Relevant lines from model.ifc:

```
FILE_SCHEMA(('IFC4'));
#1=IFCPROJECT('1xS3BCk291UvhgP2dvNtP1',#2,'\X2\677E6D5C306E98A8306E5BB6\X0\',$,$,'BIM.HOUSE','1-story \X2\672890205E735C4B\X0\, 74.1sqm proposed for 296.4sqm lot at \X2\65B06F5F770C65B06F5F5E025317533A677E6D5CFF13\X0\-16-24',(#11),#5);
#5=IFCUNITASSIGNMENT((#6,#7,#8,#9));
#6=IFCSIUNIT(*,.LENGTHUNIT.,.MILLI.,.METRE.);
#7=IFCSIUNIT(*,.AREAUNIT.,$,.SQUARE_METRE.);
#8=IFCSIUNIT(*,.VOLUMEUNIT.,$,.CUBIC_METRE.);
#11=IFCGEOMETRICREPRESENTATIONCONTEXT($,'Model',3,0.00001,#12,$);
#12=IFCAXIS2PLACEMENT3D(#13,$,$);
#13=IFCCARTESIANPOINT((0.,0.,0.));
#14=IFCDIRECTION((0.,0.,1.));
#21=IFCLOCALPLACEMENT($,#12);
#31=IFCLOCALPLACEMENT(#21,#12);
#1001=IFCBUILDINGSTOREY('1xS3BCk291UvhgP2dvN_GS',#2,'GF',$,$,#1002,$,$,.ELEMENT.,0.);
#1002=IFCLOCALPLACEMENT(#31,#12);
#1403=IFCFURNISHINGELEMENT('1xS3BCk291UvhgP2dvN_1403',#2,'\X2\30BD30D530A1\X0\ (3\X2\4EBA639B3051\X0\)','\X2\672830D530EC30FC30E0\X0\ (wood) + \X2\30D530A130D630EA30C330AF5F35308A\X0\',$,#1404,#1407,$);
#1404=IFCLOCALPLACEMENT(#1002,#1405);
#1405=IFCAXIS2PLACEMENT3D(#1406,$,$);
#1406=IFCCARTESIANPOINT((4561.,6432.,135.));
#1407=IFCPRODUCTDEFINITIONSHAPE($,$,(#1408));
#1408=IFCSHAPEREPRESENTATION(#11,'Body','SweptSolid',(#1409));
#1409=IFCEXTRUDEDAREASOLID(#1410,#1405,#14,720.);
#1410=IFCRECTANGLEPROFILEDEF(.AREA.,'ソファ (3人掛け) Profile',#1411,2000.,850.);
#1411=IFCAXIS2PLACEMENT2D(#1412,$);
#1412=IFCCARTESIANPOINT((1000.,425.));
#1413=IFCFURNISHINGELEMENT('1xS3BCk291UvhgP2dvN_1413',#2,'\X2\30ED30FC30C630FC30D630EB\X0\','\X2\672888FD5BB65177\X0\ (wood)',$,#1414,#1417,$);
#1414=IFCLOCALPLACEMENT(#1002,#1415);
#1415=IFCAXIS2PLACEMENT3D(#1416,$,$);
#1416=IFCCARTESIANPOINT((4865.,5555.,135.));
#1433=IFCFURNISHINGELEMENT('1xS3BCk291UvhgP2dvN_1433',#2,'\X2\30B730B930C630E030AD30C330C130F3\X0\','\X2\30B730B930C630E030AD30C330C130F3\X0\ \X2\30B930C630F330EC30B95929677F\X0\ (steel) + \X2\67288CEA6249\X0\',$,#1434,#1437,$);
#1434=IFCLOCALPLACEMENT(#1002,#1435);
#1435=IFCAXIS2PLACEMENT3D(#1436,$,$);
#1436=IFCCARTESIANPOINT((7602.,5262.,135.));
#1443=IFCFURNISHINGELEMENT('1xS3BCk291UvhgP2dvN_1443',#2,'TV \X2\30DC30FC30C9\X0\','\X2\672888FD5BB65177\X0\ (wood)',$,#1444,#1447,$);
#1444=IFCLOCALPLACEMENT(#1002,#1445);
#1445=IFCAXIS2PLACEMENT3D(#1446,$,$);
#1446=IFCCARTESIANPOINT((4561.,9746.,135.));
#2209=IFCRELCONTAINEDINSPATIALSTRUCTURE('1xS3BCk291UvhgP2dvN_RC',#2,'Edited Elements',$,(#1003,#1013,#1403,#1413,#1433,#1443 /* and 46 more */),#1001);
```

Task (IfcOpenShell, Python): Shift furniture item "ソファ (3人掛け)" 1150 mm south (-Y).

```python
import ifcopenshell
import ifcopenshell.api.geometry
import ifcopenshell.util.placement

model = ifcopenshell.open("model.ifc")

item = model.by_id(1403)
matrix = ifcopenshell.util.placement.get_local_placement(item.ObjectPlacement)
matrix[1, 3] -= 1150.0
ifcopenshell.api.geometry.edit_object_placement(model, product=item, matrix=matrix, is_si=False)

print(ifcopenshell.util.placement.get_local_placement(item.ObjectPlacement).round(3) + 0.0)

model.write("model_rev.ifc")
```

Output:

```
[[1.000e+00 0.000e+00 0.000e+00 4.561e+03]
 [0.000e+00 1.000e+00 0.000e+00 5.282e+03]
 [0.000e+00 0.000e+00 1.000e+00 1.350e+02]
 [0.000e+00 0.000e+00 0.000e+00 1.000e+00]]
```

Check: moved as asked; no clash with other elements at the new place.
